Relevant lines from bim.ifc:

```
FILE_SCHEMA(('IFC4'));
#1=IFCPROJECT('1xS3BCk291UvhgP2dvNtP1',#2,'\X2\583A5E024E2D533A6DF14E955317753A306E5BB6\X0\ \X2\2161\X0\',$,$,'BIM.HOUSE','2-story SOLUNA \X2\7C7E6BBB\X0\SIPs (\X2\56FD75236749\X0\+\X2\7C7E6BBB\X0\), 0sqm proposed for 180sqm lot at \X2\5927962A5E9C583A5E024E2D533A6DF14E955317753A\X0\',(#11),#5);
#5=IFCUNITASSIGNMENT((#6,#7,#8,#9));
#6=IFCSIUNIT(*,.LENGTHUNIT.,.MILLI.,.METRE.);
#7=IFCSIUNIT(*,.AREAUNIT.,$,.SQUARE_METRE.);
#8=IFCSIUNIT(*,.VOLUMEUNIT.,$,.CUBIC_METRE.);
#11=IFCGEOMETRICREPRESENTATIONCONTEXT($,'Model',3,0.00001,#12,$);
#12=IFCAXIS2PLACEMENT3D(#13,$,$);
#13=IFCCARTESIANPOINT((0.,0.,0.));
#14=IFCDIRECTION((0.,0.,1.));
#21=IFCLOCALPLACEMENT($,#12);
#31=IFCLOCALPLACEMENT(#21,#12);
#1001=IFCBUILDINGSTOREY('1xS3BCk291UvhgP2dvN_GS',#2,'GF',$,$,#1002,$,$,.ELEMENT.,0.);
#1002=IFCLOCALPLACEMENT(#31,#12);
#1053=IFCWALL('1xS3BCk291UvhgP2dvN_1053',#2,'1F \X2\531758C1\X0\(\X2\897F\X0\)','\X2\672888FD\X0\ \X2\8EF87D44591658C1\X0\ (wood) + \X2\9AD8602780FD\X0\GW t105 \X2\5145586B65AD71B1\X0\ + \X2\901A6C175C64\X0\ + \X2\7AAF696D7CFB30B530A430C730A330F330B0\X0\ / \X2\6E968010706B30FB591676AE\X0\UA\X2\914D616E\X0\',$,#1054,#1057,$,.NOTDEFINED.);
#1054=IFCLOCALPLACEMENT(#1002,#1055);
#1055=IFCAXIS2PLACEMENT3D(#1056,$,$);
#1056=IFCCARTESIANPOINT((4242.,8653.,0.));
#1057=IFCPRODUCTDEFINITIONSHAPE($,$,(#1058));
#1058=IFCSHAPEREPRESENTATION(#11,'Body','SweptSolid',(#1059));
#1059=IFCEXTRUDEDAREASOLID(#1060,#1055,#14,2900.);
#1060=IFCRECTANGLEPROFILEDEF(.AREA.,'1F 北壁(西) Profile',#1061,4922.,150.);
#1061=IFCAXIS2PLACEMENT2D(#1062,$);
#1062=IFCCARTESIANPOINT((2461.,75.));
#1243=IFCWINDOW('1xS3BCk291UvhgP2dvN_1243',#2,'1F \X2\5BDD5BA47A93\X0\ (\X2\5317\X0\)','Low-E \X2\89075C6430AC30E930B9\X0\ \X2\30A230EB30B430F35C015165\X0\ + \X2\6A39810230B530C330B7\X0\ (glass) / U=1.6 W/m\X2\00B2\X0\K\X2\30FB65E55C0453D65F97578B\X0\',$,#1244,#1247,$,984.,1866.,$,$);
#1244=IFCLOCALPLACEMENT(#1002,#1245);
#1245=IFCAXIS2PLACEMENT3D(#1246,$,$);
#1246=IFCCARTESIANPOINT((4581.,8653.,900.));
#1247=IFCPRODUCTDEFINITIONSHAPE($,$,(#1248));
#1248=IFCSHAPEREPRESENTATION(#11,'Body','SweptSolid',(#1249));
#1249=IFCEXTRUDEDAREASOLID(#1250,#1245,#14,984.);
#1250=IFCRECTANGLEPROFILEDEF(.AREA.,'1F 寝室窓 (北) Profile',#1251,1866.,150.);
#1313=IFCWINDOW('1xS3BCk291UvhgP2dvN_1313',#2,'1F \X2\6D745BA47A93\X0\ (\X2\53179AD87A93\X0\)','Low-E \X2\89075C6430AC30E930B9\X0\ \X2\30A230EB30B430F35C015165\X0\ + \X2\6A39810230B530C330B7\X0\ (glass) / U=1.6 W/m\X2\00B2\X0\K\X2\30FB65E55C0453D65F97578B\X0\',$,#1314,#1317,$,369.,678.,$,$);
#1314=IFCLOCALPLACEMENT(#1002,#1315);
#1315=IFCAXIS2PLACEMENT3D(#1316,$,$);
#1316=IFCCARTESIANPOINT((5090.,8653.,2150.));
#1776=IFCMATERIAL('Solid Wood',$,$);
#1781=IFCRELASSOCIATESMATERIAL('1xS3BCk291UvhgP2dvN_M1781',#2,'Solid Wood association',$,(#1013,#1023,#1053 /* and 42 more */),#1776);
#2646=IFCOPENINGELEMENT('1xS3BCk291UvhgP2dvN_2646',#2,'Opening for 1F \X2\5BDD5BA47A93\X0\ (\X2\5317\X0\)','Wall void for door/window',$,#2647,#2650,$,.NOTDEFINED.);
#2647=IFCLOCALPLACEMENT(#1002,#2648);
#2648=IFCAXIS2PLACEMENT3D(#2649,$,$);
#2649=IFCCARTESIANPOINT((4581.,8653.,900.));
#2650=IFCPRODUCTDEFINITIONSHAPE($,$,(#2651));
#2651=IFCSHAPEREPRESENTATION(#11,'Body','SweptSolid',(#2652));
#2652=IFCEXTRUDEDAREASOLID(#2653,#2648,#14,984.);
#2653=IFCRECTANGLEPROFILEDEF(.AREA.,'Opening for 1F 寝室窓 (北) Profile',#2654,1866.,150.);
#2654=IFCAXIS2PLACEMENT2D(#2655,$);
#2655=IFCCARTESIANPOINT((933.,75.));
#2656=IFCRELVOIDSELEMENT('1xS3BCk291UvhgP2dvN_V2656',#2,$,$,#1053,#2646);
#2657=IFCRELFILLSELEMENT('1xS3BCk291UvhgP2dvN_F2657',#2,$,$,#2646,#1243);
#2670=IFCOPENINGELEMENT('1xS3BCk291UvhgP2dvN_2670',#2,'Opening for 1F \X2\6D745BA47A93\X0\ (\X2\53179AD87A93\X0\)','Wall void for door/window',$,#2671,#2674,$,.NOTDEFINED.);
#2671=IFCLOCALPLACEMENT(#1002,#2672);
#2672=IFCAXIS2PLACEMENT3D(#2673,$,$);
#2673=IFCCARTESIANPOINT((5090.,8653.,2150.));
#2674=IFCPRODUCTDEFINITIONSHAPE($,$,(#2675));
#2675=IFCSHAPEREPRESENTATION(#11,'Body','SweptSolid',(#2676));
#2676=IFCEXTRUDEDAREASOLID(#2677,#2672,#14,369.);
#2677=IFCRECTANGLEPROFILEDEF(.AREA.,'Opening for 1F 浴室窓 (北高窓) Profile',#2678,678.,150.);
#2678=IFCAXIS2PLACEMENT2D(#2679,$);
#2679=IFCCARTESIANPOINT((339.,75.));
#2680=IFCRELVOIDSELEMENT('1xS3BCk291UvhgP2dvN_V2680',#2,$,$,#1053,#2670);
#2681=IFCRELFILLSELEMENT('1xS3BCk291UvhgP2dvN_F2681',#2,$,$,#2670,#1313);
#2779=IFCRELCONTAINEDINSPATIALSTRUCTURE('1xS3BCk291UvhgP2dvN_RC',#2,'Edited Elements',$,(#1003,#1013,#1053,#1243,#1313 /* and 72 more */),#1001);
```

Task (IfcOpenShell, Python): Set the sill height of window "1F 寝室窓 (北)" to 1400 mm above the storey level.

```python
import numpy as np
import ifcopenshell
import ifcopenshell.api.geometry
import ifcopenshell.geom
import ifcopenshell.util.element
import ifcopenshell.util.placement
import ifcopenshell.util.shape
import ifcopenshell.util.unit

model = ifcopenshell.open("bim.ifc")
unit_scale = ifcopenshell.util.unit.calculate_unit_scale(model)

window = model.by_guid("1xS3BCk291UvhgP2dvN_1243")
opening = window.FillsVoids[0].RelatingOpeningElement
storey = ifcopenshell.util.element.get_container(window, ifc_class="IfcBuildingStorey")
level = ifcopenshell.util.placement.get_local_placement(storey.ObjectPlacement)[2, 3]

# The opening's origin need not be at the sill, so measure its lowest point.
shape = ifcopenshell.geom.create_shape(ifcopenshell.geom.settings(), opening)
bottom = ifcopenshell.util.shape.get_shape_bottom_elevation(shape, shape.geometry) / unit_scale
dz = level + 1.4 / unit_scale - bottom

shift = np.array([0.0, 0.0, dz])
# The window is not placed relative to its opening, so move both.
for product in (opening, window):
    matrix = ifcopenshell.util.placement.get_local_placement(product.ObjectPlacement)
    matrix[:3, 3] += shift
    ifcopenshell.api.geometry.edit_object_placement(model, product=product, matrix=matrix, is_si=False)

print(f"moved by {dz * unit_scale:+.3f} m")

model.write("bim_v2.ifc")
```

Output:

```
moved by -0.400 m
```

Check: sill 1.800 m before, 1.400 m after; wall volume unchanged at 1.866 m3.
